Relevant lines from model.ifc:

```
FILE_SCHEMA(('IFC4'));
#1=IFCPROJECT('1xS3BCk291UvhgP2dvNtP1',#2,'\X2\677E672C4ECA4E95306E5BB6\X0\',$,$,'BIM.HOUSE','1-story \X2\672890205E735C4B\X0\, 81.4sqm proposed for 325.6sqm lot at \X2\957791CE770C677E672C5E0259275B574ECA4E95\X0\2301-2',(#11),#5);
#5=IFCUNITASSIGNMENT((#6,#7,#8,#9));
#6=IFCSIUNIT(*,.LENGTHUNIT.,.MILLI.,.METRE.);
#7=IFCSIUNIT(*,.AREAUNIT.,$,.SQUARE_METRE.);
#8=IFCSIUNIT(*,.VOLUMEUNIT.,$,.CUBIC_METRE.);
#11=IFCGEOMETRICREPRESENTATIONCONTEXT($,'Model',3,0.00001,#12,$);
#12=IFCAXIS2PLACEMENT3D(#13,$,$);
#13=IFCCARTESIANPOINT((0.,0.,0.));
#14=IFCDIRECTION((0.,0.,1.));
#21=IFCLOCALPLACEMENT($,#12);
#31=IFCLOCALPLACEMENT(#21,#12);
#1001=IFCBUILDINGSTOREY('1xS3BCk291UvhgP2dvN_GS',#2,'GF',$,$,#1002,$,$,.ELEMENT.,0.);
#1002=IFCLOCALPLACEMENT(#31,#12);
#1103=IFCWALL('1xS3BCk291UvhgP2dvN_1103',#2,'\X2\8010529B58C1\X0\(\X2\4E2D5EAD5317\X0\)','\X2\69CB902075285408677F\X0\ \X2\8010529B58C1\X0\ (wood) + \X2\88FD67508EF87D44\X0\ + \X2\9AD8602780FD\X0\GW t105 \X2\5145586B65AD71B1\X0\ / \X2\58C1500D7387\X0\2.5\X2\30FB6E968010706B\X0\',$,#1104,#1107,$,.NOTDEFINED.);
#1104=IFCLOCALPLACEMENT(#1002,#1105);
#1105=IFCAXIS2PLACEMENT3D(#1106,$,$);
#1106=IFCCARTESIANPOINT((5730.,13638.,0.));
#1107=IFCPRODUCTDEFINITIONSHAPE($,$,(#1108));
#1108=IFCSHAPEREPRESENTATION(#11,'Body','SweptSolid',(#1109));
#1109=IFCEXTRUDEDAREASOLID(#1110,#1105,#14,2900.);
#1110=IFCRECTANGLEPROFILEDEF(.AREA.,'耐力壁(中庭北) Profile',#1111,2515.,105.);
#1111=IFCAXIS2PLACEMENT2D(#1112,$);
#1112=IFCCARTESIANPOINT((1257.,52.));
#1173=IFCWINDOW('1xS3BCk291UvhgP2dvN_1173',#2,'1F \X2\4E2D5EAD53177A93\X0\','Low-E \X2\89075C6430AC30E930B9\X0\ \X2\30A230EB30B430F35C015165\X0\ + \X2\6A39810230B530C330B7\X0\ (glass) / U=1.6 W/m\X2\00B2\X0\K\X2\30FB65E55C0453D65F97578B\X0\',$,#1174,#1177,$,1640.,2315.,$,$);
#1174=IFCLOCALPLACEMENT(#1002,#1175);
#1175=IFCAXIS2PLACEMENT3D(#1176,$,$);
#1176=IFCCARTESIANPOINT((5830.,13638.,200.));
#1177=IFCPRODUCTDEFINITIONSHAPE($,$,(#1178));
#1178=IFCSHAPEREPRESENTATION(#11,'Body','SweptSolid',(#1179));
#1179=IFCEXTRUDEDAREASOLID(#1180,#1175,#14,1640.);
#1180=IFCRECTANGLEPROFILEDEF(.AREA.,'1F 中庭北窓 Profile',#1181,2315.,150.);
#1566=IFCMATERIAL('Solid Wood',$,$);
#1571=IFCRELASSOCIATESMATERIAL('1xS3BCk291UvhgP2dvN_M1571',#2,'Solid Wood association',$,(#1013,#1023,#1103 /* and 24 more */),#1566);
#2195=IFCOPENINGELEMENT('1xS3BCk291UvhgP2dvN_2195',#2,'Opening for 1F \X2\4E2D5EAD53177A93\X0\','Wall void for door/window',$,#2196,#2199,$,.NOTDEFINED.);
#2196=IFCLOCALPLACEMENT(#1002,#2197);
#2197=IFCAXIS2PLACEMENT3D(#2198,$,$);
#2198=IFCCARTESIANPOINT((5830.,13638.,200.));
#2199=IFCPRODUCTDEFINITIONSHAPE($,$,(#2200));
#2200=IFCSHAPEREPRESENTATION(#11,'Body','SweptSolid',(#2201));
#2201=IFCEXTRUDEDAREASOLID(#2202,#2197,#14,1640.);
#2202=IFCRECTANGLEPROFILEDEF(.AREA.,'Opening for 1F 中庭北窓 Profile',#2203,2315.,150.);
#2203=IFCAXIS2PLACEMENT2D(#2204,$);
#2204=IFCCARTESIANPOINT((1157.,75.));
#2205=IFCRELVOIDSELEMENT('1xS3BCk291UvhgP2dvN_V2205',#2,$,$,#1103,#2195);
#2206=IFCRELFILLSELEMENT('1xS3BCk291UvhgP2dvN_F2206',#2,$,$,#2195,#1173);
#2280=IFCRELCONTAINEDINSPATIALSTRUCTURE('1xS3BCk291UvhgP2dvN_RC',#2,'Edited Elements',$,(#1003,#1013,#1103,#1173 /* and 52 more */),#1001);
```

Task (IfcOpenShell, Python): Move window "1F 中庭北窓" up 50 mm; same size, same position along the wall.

```python
import numpy as np
import ifcopenshell
import ifcopenshell.api.geometry
import ifcopenshell.util.placement
import ifcopenshell.util.unit

model = ifcopenshell.open("model.ifc")
unit_scale = ifcopenshell.util.unit.calculate_unit_scale(model)

window = model.by_guid("1xS3BCk291UvhgP2dvN_1173")
opening = window.FillsVoids[0].RelatingOpeningElement
dz = 50.0

shift = np.array([0.0, 0.0, dz])
# The window is not placed relative to its opening, so move both.
for product in (opening, window):
    matrix = ifcopenshell.util.placement.get_local_placement(product.ObjectPlacement)
    matrix[:3, 3] += shift
    ifcopenshell.api.geometry.edit_object_placement(model, product=product, matrix=matrix, is_si=False)

print(f"moved by {dz * unit_scale:+.3f} m")

model.write("model-out.ifc")
```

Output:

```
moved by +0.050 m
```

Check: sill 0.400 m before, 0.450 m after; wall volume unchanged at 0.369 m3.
